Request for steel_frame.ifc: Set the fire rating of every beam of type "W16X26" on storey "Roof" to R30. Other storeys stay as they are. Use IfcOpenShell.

First a look at what the model holds.

```python
import ifcopenshell
import ifcopenshell.util.element

model = ifcopenshell.open("steel_frame.ifc")
print(model.schema)
storey = next(s for s in model.by_type("IfcBuildingStorey") if s.Name == "Roof")
beams = [e for e in ifcopenshell.util.element.get_decomposition(storey) if e.is_a("IfcBeam")]
seen = {}
for e in beams:
    element_type = ifcopenshell.util.element.get_type(e)
    key = (element_type.Name if element_type != e and element_type else None, ifcopenshell.util.element.get_pset(e, "Pset_BeamCommon", "FireRating"))
    seen[key] = seen.get(key, 0) + 1
for (name, value), count in sorted(seen.items(), key=str):
    print(count, "x", name, "|", value)
```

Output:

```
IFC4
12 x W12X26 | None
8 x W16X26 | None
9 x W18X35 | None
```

```python
import ifcopenshell
import ifcopenshell.api.pset
import ifcopenshell.util.element

model = ifcopenshell.open("steel_frame.ifc")

storey = next(s for s in model.by_type("IfcBuildingStorey") if s.Name == "Roof")
beams = [e for e in ifcopenshell.util.element.get_decomposition(storey) if e.is_a("IfcBeam")]

count = 0
for e in beams:
    element_type = ifcopenshell.util.element.get_type(e)
    if element_type in (None, e) or element_type.Name != "W16X26":
        continue
    # add_pset returns the element's existing set when there is one.
    pset = ifcopenshell.api.pset.add_pset(model, product=e, name="Pset_BeamCommon")
    ifcopenshell.api.pset.edit_pset(model, pset=pset, properties={"FireRating": "R30"})
    count += 1

print(count, "beams updated")

model.write("steel_frame_updated.ifc")
```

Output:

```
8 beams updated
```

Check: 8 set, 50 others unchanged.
